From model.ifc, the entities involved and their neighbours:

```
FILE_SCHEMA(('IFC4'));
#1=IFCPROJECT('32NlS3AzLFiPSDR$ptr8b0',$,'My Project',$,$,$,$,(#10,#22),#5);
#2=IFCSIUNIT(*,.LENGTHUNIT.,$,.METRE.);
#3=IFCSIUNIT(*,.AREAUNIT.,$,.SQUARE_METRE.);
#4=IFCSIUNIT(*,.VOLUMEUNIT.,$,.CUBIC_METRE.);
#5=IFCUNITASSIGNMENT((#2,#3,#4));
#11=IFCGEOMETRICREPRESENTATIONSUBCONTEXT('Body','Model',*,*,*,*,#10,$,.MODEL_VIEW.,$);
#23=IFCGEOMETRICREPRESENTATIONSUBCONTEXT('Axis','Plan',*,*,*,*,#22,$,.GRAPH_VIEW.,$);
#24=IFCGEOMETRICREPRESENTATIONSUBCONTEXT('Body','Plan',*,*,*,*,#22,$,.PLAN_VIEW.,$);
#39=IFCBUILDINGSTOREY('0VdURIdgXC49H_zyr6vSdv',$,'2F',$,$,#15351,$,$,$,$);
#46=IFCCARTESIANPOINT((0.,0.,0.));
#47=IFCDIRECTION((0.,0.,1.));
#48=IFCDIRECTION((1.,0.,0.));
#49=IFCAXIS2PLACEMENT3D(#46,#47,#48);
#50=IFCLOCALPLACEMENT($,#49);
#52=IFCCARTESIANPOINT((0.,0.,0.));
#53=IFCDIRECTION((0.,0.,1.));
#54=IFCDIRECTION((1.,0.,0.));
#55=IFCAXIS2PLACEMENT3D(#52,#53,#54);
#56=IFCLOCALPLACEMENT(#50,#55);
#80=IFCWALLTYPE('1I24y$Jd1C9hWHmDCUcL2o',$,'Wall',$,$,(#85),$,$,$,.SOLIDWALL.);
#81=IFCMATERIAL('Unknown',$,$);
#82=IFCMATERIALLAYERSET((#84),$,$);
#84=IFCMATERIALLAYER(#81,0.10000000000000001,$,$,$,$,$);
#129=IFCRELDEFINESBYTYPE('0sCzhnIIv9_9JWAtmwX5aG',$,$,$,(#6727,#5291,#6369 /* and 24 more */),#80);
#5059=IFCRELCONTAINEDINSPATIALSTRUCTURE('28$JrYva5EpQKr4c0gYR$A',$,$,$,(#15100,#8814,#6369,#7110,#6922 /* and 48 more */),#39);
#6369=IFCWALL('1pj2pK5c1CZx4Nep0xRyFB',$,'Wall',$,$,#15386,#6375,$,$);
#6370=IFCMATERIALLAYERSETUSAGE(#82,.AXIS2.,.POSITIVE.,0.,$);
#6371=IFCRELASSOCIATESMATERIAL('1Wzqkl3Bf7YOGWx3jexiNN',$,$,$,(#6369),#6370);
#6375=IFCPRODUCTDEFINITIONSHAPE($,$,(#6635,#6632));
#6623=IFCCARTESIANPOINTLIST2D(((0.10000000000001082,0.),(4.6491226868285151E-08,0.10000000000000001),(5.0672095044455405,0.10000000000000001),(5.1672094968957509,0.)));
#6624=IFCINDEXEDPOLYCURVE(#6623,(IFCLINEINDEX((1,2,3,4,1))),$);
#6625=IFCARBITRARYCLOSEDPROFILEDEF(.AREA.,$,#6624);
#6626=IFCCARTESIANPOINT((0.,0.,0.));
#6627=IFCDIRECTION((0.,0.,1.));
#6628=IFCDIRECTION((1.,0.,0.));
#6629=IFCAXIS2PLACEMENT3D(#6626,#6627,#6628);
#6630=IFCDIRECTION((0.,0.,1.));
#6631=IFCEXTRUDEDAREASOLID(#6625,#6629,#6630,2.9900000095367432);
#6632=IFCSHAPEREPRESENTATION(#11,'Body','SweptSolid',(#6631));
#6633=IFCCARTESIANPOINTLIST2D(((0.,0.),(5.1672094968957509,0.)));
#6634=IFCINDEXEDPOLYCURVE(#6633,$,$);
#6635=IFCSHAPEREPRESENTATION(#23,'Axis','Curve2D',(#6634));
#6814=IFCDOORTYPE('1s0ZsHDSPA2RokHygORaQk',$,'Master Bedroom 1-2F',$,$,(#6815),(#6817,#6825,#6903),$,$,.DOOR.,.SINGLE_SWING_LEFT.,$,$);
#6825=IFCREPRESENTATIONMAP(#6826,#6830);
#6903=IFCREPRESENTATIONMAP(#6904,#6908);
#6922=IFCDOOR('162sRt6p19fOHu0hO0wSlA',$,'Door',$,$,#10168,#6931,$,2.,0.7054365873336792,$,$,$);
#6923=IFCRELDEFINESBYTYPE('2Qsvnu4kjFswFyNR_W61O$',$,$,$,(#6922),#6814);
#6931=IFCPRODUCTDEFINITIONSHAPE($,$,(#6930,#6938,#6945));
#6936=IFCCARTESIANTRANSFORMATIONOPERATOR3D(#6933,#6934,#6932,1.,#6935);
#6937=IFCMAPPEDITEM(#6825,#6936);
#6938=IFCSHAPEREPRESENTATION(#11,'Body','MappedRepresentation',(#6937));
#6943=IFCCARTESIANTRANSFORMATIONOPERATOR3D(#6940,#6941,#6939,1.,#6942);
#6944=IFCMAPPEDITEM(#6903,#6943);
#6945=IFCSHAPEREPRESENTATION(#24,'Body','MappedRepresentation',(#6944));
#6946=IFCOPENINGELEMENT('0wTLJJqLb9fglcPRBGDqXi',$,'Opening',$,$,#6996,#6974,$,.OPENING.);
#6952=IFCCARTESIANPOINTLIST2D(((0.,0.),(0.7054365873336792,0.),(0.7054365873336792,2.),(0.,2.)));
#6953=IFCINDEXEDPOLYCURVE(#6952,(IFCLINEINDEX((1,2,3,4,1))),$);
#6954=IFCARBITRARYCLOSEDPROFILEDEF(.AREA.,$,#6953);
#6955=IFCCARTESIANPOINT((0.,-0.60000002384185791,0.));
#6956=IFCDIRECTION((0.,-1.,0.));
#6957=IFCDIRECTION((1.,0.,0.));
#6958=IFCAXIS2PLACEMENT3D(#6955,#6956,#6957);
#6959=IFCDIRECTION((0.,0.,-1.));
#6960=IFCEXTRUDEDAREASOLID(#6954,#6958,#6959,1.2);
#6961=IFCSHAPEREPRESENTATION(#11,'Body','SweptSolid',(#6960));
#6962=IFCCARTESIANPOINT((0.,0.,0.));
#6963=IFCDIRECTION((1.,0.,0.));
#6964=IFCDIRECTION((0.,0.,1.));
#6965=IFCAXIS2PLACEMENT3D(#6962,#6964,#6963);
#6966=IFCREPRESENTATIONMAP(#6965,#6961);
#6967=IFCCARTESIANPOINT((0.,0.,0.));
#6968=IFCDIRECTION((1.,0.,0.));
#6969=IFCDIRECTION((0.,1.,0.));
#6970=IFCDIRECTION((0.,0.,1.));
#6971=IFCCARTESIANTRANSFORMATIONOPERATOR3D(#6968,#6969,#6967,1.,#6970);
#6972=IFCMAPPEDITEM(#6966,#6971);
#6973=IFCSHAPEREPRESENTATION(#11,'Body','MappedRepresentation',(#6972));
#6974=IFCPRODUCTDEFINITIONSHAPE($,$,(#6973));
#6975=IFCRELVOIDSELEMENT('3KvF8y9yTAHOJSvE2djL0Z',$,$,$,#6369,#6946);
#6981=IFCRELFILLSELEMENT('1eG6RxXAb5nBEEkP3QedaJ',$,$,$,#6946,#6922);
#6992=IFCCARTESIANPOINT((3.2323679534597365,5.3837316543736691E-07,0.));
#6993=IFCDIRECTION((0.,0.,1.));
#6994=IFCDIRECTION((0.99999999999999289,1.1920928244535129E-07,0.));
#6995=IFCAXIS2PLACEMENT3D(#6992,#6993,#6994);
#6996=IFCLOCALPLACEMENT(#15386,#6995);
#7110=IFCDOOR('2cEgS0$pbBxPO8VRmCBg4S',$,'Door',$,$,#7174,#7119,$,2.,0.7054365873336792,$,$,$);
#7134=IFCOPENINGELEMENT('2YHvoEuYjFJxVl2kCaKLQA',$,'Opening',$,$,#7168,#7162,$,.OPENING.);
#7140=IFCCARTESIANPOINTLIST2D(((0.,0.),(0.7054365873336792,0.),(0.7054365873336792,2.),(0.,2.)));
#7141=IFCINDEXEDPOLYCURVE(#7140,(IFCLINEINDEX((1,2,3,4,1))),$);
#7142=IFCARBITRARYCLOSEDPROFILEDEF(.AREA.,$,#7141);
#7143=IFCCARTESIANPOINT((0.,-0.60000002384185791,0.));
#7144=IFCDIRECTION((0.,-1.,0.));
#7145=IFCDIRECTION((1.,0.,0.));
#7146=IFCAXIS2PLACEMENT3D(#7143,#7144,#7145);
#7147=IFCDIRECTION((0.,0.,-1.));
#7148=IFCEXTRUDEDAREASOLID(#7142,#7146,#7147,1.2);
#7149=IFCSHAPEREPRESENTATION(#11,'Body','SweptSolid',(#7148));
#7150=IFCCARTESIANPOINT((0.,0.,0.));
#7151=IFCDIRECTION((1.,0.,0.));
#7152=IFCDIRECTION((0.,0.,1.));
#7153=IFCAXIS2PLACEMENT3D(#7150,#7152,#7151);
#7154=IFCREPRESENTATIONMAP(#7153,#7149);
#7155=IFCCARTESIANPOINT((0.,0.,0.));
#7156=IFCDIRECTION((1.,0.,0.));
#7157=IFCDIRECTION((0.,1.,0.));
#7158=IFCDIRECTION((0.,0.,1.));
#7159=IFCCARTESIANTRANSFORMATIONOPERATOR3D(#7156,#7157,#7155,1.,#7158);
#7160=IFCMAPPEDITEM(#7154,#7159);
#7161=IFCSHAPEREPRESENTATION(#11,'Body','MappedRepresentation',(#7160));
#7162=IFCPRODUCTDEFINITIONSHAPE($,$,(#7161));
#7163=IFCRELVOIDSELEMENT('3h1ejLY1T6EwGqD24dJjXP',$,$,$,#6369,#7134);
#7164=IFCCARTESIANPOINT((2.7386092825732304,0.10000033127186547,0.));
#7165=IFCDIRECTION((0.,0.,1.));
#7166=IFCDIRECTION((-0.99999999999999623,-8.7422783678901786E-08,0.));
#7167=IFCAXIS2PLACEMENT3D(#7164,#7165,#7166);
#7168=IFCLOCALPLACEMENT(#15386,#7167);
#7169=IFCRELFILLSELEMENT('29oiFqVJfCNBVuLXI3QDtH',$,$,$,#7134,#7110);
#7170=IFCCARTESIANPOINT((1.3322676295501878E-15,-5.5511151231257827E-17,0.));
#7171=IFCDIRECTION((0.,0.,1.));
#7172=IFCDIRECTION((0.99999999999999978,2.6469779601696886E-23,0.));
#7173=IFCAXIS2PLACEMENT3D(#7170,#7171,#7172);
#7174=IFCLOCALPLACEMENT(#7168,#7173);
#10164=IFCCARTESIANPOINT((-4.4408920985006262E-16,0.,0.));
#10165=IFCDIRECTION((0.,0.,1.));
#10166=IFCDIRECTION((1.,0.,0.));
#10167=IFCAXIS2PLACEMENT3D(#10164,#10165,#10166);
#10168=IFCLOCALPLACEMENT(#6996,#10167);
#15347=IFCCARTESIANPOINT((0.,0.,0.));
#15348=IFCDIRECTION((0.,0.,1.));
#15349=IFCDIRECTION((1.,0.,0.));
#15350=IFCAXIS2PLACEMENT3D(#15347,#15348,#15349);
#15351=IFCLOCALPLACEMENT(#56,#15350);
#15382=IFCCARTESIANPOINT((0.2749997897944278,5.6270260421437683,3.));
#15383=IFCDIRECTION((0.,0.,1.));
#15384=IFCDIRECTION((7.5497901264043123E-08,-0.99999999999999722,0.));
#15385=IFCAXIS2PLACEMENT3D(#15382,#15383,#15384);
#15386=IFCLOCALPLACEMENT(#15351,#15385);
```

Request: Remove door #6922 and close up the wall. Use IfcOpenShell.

```python
import ifcopenshell
import ifcopenshell.api.feature
import ifcopenshell.api.root
import ifcopenshell.geom
import ifcopenshell.util.shape

model = ifcopenshell.open("model.ifc")
settings = ifcopenshell.geom.settings()


def volume(element):
    """Net volume in cubic metres, openings subtracted."""
    shape = ifcopenshell.geom.create_shape(settings, element)
    return ifcopenshell.util.shape.get_volume(shape.geometry)


door = model.by_id(6922)
opening = door.FillsVoids[0].RelatingOpeningElement
wall = opening.VoidsElements[0].RelatingBuildingElement
before = volume(wall)

ifcopenshell.api.root.remove_product(model, product=door)
ifcopenshell.api.feature.remove_feature(model, feature=opening)

after = volume(wall)

print(f"wall volume {before:.3f} -> {after:.3f} m3")

model.write("model_updated.ifc")
```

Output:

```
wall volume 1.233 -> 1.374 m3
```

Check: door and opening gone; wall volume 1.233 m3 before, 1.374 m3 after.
